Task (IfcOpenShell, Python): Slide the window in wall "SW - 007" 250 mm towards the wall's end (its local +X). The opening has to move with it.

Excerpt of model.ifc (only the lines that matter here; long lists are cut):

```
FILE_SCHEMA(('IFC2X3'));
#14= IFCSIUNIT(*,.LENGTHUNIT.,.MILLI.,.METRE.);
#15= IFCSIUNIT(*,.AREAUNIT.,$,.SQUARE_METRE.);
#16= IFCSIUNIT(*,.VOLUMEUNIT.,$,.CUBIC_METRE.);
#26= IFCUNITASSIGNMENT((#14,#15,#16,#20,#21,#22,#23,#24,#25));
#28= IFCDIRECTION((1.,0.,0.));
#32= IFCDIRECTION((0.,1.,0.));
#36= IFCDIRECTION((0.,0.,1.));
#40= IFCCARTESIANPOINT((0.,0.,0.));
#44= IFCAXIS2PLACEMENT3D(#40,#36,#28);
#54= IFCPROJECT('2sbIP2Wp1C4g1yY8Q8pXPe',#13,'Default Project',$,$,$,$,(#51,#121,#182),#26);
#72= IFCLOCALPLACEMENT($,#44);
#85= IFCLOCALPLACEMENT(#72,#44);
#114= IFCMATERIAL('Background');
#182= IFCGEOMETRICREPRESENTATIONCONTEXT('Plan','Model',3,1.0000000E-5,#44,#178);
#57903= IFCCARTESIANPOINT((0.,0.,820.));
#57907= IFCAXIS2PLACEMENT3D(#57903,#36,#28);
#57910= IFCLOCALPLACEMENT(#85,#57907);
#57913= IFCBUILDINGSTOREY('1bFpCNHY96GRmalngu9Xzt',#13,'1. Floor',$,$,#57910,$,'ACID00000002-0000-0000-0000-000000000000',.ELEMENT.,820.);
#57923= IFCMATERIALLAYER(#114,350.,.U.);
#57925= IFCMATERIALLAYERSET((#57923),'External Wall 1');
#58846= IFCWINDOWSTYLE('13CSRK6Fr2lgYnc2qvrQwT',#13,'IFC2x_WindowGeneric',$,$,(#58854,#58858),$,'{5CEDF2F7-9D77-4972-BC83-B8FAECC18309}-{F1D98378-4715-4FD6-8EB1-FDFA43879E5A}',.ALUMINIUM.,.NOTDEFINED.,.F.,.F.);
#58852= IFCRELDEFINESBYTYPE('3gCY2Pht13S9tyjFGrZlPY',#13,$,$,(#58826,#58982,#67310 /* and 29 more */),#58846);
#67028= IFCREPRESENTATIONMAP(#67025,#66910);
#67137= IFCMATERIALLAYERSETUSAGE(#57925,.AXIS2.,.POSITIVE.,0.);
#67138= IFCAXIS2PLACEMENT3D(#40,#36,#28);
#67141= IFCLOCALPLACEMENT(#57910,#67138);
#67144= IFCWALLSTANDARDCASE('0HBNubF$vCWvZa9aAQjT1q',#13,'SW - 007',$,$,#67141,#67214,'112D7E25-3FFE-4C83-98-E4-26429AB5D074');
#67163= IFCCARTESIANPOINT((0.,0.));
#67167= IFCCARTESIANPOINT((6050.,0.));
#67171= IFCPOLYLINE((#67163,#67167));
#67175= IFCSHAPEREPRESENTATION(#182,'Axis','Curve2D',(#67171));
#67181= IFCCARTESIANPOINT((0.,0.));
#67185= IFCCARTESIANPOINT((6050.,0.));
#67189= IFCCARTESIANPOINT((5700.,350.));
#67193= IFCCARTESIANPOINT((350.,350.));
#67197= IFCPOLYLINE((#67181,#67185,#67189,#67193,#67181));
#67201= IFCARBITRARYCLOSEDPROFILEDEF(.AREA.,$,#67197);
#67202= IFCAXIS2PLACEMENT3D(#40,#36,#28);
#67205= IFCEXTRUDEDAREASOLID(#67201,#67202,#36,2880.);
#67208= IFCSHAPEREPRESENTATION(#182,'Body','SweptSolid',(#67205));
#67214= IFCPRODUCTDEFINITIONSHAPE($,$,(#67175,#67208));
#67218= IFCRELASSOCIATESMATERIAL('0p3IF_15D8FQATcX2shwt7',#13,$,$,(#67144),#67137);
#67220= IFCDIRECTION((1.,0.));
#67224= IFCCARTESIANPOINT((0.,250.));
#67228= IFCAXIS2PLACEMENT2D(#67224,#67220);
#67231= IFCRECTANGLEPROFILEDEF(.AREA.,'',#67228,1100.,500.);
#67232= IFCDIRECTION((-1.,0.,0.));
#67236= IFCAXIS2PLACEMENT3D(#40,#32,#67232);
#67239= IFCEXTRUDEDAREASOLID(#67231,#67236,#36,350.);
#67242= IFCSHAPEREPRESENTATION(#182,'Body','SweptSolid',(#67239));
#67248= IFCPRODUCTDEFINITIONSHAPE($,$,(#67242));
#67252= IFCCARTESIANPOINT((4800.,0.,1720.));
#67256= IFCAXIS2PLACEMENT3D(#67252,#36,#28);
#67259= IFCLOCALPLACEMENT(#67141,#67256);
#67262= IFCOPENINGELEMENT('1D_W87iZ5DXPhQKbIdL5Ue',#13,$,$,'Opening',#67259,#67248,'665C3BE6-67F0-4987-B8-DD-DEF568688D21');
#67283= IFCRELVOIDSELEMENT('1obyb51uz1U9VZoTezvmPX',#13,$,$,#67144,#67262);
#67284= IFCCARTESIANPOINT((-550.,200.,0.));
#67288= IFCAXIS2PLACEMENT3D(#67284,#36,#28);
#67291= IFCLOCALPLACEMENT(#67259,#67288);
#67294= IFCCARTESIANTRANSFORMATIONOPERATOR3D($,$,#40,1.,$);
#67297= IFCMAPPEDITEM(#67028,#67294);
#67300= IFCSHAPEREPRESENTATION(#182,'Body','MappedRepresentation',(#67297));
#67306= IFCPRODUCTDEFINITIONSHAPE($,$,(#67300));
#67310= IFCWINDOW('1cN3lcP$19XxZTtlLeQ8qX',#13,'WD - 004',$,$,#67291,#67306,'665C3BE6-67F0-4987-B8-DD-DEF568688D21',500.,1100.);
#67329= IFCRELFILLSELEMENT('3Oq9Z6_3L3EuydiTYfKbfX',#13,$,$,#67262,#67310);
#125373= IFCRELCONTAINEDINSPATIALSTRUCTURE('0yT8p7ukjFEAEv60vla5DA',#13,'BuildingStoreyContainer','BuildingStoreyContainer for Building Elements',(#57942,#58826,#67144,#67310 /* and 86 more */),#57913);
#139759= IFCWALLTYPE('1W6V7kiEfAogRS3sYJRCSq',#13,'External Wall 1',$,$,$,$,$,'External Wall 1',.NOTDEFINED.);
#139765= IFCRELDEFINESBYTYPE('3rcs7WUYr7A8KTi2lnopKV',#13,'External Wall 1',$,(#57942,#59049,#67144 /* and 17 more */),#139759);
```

```python
import ifcopenshell
import ifcopenshell.api.geometry
import ifcopenshell.util.placement
import ifcopenshell.util.unit

model = ifcopenshell.open("model.ifc")
unit_scale = ifcopenshell.util.unit.calculate_unit_scale(model)

window = model.by_id(67310)
opening = window.FillsVoids[0].RelatingOpeningElement
wall = opening.VoidsElements[0].RelatingBuildingElement

wall_matrix = ifcopenshell.util.placement.get_local_placement(wall.ObjectPlacement)
shift = wall_matrix[:3, 0] * 0.25 / unit_scale
before = ifcopenshell.util.placement.get_local_placement(window.ObjectPlacement)[:3, 3].copy()

# The window is placed relative to its opening, so it follows when the opening moves.
matrix = ifcopenshell.util.placement.get_local_placement(opening.ObjectPlacement)
matrix[:3, 3] += shift
ifcopenshell.api.geometry.edit_object_placement(
    model, product=opening, matrix=matrix, is_si=False, should_transform_children=True
)

after = ifcopenshell.util.placement.get_local_placement(window.ObjectPlacement)[:3, 3]
print("window moved by", (after - before).round(3) + 0.0)

model.write("model_edited.ifc")
```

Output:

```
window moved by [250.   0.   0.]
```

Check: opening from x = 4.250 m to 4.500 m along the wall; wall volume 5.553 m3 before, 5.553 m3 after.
